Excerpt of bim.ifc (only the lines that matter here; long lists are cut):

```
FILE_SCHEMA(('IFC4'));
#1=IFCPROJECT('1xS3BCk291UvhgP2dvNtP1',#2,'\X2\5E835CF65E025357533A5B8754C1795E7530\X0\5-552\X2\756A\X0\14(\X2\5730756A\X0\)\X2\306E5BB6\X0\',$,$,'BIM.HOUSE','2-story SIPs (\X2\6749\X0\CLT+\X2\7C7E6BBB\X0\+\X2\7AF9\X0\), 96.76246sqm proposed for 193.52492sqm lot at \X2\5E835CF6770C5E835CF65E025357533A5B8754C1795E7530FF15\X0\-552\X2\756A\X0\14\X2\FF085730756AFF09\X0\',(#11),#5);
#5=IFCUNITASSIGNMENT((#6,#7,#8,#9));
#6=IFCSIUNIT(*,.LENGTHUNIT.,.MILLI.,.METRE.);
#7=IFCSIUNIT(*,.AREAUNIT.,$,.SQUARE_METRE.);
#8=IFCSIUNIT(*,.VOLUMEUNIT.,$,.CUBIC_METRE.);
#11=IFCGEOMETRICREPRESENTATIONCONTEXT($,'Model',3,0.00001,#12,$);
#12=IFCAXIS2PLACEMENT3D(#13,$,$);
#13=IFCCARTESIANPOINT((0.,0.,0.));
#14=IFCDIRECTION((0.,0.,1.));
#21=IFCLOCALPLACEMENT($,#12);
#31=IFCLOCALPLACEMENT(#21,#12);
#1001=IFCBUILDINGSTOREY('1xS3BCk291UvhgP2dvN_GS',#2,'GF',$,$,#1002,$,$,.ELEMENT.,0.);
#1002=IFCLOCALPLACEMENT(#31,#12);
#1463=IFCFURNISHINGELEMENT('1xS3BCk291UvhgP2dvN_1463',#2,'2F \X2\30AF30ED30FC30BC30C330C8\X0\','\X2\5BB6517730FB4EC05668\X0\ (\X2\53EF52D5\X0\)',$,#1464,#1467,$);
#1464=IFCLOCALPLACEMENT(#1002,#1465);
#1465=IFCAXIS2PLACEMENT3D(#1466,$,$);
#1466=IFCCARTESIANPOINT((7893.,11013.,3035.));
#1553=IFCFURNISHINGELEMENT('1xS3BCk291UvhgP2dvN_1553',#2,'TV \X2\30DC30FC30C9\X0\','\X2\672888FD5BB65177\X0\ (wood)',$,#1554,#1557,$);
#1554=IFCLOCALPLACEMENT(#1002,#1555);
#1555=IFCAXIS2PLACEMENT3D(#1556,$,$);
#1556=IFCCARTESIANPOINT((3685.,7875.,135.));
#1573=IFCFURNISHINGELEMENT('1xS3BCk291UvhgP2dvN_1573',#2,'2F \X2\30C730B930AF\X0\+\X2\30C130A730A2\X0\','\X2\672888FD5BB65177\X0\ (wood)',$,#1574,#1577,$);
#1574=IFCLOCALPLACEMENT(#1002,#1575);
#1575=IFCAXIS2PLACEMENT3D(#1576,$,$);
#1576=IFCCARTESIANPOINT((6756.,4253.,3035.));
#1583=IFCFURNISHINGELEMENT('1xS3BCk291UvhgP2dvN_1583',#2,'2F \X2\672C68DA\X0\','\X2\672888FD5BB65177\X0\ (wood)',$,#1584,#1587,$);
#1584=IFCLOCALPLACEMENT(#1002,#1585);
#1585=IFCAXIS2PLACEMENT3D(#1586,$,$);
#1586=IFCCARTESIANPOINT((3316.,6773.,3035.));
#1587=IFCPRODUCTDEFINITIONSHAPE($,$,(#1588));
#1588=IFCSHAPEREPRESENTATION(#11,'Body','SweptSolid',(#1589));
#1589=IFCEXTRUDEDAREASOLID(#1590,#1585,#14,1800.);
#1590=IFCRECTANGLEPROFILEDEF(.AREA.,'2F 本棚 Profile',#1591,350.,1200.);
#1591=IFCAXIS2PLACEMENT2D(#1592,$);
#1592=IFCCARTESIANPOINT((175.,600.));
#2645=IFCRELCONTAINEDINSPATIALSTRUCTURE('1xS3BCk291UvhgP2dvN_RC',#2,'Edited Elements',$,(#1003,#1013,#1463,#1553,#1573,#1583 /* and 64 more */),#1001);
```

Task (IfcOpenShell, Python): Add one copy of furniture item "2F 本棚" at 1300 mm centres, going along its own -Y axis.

```python
import ifcopenshell
import ifcopenshell.api.geometry
import ifcopenshell.api.root
import ifcopenshell.util.element
import ifcopenshell.util.placement
import ifcopenshell.util.unit

model = ifcopenshell.open("bim.ifc")
unit_scale = ifcopenshell.util.unit.calculate_unit_scale(model)


def reuse_history(source, copy):
    """copy_class also copies each property set's owner history, people and application; keep the originals."""
    for rel in copy.IsDefinedBy:
        if rel.is_a("IfcRelDefinesByProperties") and (history := rel.RelatingPropertyDefinition.OwnerHistory):
            rel.RelatingPropertyDefinition.OwnerHistory = source.OwnerHistory
            ifcopenshell.util.element.remove_deep2(model, history)


source = model.by_guid("1xS3BCk291UvhgP2dvN_1583")
base = ifcopenshell.util.placement.get_local_placement(source.ObjectPlacement)
step = -base[:3, 1] * 1.3 / unit_scale

for i in range(1, 2):
    copy = ifcopenshell.api.root.copy_class(model, product=source)
    copy.Representation = ifcopenshell.util.element.copy_deep(
        model, source.Representation, exclude=["IfcGeometricRepresentationContext", "IfcRepresentationMap"]
    )
    reuse_history(source, copy)
    matrix = base.copy()
    matrix[:3, 3] += i * step
    print("added at", matrix[:3, 3].round(3) + 0.0)
    ifcopenshell.api.geometry.edit_object_placement(model, product=copy, matrix=matrix, is_si=False)

model.write("bim_edited.ifc")
```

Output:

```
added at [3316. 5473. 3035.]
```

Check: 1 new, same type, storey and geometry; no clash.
